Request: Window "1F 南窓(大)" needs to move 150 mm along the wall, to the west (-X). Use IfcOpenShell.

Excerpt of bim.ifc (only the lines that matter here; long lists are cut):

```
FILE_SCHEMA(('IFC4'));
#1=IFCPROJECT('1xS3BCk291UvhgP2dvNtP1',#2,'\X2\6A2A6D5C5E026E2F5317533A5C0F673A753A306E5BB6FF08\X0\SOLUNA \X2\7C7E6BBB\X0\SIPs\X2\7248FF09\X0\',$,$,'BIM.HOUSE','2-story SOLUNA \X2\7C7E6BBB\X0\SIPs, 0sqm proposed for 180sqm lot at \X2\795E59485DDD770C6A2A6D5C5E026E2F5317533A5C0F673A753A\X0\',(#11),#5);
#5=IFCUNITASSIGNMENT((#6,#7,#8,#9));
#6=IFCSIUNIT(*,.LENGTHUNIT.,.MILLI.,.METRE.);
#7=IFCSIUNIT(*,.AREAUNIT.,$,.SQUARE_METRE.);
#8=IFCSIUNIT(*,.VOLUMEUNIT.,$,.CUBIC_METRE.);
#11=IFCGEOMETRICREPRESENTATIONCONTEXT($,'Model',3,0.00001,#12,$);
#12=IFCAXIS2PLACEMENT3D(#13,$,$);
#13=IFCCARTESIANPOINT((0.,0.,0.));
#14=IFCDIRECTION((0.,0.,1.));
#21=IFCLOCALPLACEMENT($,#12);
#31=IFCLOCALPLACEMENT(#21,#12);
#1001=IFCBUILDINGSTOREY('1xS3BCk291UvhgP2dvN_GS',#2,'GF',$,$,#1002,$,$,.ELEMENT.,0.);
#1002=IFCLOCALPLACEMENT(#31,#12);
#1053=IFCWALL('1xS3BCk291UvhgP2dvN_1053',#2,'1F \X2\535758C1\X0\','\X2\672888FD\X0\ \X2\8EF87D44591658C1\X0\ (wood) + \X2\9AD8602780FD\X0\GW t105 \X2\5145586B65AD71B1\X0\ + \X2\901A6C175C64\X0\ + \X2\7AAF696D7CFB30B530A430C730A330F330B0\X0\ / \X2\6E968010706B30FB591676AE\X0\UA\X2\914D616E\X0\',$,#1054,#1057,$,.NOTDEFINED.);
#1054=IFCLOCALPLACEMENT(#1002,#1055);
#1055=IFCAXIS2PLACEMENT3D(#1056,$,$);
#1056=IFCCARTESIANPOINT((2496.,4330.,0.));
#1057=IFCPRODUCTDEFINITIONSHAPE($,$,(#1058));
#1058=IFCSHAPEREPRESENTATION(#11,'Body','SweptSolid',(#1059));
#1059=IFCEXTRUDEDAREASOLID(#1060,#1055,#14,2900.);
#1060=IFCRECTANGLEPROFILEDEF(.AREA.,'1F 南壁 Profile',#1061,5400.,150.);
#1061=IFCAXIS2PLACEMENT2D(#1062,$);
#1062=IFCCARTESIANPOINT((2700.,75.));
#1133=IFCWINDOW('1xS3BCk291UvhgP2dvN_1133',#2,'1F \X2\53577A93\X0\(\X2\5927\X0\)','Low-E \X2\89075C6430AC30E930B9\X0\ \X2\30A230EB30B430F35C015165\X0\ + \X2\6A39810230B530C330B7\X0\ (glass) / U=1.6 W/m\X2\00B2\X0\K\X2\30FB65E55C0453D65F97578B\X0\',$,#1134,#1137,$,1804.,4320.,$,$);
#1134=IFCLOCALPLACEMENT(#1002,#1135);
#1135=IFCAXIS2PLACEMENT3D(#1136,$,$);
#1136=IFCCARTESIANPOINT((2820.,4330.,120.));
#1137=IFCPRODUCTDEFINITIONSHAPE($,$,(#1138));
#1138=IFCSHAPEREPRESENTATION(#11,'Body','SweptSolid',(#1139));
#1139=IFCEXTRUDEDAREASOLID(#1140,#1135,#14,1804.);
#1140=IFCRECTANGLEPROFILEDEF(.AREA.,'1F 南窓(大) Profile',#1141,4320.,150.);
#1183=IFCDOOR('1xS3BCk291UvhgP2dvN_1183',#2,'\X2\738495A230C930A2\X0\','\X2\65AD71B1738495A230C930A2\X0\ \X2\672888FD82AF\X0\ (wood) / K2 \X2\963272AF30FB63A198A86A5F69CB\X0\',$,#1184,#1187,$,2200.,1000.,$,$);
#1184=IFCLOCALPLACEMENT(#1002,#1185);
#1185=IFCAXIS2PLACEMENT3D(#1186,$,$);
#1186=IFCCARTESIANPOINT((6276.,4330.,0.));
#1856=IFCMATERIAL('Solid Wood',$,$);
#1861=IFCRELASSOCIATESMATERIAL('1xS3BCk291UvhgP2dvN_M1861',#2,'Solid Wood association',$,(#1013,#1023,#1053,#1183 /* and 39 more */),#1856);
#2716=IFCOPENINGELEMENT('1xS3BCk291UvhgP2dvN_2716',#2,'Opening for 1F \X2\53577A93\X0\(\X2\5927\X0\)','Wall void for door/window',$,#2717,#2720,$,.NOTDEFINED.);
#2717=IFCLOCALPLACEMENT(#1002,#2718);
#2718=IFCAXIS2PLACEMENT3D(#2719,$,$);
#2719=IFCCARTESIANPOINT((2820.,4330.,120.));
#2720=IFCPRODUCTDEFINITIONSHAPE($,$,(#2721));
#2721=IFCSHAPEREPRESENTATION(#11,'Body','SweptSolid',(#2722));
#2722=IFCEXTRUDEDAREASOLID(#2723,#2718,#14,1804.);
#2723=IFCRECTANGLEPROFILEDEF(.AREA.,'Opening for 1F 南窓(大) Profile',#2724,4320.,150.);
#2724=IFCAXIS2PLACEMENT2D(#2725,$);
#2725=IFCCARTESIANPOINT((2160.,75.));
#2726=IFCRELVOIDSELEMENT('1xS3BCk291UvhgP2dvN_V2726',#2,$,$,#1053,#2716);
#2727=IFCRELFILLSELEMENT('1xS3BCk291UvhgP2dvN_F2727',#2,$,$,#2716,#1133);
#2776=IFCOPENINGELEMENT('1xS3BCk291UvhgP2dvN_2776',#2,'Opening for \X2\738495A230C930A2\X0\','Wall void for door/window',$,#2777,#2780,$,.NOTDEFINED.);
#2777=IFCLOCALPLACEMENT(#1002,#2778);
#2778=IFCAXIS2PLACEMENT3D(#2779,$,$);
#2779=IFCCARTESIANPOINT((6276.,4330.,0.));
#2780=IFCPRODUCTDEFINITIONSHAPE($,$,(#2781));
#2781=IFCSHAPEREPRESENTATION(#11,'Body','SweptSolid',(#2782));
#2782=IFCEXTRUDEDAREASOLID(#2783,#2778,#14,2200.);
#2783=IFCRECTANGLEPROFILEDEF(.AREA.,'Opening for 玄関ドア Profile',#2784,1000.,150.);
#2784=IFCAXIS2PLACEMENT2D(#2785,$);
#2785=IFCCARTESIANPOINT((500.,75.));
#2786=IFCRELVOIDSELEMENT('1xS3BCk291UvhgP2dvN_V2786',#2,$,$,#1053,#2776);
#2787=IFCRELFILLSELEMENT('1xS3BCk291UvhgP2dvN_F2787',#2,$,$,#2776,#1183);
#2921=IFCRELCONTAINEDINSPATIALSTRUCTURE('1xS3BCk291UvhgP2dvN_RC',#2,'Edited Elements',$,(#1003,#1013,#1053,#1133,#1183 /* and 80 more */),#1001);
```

```python
import ifcopenshell
import ifcopenshell.api.geometry
import ifcopenshell.util.placement

model = ifcopenshell.open("bim.ifc")

window = model.by_id(1133)
opening = window.FillsVoids[0].RelatingOpeningElement
wall = opening.VoidsElements[0].RelatingBuildingElement

wall_matrix = ifcopenshell.util.placement.get_local_placement(wall.ObjectPlacement)
shift = wall_matrix[:3, 0] * -150.0
before = ifcopenshell.util.placement.get_local_placement(window.ObjectPlacement)[:3, 3].copy()

# The window is not placed relative to its opening, so move both.
for product in (opening, window):
    matrix = ifcopenshell.util.placement.get_local_placement(product.ObjectPlacement)
    matrix[:3, 3] += shift
    ifcopenshell.api.geometry.edit_object_placement(model, product=product, matrix=matrix, is_si=False)

after = ifcopenshell.util.placement.get_local_placement(window.ObjectPlacement)[:3, 3]
print("window moved by", (after - before).round(3) + 0.0)

model.write("bim_v2.ifc")
```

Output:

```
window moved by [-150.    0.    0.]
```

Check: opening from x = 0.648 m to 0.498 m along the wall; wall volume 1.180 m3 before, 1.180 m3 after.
